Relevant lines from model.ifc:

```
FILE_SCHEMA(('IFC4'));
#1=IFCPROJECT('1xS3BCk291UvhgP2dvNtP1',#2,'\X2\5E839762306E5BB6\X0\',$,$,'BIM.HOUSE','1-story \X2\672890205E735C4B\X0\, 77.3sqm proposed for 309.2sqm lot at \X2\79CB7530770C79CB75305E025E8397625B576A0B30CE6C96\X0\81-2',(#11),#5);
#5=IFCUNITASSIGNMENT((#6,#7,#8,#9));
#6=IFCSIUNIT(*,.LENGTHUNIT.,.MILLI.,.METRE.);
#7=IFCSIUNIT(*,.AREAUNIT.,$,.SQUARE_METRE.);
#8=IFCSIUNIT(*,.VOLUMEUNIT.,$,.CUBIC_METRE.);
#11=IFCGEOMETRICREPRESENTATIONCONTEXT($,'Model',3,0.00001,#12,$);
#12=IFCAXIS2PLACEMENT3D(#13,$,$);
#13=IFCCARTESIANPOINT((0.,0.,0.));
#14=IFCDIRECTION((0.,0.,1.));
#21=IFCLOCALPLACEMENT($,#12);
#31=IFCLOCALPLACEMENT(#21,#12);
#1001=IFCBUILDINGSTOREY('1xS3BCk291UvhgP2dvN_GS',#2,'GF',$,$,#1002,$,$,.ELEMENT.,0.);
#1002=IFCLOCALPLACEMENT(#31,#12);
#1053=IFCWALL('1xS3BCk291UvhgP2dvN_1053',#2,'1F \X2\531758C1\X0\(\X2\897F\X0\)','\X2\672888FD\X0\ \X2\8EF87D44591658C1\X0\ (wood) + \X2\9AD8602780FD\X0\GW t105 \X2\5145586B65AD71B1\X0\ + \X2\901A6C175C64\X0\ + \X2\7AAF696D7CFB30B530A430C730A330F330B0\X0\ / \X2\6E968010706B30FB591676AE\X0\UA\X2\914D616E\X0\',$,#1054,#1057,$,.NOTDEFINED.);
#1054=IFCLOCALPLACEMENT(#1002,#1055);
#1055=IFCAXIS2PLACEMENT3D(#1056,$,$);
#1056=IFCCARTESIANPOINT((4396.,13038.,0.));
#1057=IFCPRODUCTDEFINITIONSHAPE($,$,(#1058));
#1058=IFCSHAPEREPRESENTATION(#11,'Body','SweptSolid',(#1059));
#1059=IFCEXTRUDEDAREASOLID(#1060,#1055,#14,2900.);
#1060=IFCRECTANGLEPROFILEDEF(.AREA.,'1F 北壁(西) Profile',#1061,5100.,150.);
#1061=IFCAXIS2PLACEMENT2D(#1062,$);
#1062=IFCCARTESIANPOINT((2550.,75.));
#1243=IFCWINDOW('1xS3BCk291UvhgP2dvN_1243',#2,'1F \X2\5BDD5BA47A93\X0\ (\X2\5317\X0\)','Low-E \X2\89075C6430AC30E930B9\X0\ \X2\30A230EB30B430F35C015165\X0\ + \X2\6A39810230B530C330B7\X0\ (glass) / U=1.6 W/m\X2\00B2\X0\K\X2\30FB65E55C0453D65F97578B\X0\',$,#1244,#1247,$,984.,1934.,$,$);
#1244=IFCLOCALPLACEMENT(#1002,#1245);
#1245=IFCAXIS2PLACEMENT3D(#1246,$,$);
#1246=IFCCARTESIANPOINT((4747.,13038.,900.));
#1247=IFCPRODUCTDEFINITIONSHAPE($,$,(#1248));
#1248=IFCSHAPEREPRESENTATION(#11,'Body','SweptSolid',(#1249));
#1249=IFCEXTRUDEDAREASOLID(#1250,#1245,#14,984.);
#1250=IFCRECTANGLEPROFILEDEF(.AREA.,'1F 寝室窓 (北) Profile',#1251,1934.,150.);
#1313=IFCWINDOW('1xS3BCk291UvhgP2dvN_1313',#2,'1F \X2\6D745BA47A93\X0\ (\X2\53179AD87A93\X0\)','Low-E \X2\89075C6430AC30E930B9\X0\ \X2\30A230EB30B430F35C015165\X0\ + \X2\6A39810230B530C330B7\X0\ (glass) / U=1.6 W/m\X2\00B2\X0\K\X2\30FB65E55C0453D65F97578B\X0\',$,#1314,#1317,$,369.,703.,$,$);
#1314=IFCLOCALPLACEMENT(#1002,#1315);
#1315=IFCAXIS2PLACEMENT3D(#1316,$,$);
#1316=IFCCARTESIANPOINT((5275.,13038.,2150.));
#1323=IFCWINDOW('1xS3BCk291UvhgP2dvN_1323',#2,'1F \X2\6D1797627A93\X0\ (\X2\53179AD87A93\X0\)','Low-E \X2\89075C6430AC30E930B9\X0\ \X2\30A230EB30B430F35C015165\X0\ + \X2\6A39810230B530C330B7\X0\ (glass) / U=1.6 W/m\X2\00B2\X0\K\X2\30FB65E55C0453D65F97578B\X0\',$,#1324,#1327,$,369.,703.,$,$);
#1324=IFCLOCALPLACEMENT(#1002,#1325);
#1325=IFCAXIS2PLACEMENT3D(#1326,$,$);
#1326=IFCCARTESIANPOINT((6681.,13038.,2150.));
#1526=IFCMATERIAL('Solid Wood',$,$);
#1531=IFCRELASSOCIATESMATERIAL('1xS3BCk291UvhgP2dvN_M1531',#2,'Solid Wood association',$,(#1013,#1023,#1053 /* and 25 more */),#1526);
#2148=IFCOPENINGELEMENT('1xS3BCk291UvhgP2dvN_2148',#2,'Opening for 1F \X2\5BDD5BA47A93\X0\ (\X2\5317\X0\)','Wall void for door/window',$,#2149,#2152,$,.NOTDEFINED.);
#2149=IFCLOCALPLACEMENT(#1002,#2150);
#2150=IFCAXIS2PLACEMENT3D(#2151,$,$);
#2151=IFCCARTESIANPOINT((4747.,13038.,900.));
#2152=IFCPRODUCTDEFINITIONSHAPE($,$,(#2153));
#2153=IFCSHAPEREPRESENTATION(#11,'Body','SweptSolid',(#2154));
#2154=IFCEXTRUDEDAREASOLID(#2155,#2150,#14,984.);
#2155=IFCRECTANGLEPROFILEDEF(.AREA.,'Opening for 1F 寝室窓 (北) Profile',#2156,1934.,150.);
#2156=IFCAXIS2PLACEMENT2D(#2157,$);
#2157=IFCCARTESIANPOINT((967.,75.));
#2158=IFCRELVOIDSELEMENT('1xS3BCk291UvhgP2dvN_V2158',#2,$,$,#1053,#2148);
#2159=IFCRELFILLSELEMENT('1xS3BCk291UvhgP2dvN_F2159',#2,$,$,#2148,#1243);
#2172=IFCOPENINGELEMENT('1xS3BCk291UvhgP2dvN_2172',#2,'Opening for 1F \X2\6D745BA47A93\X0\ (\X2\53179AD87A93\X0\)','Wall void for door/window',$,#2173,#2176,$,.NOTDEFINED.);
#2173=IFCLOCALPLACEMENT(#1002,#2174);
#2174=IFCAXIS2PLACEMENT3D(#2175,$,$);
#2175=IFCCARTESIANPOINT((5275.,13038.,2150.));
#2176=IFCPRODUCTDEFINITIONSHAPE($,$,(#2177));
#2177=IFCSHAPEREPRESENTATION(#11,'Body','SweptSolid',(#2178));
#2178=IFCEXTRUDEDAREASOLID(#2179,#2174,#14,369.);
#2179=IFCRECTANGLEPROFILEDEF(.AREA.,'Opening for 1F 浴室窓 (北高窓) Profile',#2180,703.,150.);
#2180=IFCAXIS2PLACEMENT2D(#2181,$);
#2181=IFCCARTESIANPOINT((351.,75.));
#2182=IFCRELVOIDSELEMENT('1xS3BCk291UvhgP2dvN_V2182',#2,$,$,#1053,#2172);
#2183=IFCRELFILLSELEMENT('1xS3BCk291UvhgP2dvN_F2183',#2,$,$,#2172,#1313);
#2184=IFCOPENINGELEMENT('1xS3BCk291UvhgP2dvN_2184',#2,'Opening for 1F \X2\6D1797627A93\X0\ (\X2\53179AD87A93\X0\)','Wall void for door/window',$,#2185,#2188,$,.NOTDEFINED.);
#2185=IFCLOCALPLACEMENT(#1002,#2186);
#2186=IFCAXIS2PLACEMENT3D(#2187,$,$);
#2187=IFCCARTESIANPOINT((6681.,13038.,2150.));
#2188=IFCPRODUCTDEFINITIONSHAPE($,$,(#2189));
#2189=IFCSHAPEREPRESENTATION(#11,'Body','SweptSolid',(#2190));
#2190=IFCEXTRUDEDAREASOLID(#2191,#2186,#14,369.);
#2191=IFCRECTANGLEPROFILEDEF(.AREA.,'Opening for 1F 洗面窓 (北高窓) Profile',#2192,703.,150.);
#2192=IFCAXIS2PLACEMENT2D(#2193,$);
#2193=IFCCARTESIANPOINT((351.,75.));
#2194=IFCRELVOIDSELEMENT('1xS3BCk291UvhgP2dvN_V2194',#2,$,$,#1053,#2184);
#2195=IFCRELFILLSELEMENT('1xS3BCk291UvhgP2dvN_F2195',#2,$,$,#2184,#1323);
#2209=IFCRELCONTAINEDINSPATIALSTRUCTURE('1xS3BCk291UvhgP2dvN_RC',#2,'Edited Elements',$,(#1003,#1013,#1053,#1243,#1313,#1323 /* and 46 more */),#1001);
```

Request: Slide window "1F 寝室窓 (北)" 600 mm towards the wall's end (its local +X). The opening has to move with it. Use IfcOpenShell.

```python
import ifcopenshell
import ifcopenshell.api.geometry
import ifcopenshell.util.placement

model = ifcopenshell.open("model.ifc")

window = model.by_guid("1xS3BCk291UvhgP2dvN_1243")
opening = window.FillsVoids[0].RelatingOpeningElement
wall = opening.VoidsElements[0].RelatingBuildingElement

wall_matrix = ifcopenshell.util.placement.get_local_placement(wall.ObjectPlacement)
shift = wall_matrix[:3, 0] * 600.0
before = ifcopenshell.util.placement.get_local_placement(window.ObjectPlacement)[:3, 3].copy()

# The window is not placed relative to its opening, so move both.
for product in (opening, window):
    matrix = ifcopenshell.util.placement.get_local_placement(product.ObjectPlacement)
    matrix[:3, 3] += shift
    ifcopenshell.api.geometry.edit_object_placement(model, product=product, matrix=matrix, is_si=False)

after = ifcopenshell.util.placement.get_local_placement(window.ObjectPlacement)[:3, 3]
print("window moved by", (after - before).round(3) + 0.0)

model.write("model-out.ifc")
```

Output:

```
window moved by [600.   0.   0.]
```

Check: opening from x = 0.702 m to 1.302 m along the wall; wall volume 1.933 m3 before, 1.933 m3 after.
